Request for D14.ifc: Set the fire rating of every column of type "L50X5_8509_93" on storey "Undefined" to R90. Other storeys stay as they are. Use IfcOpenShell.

First a look at what the model holds.

```python
import ifcopenshell
import ifcopenshell.util.element

model = ifcopenshell.open("D14.ifc")
print(model.schema)
storey = next(s for s in model.by_type("IfcBuildingStorey") if s.Name == "Undefined")
columns = [e for e in ifcopenshell.util.element.get_decomposition(storey) if e.is_a("IfcColumn")]
seen = {}
for e in columns:
    element_type = ifcopenshell.util.element.get_type(e)
    key = (element_type.Name if element_type != e and element_type else None, ifcopenshell.util.element.get_pset(e, "Pset_ColumnCommon", "FireRating"))
    seen[key] = seen.get(key, 0) + 1
for (name, value), count in sorted(seen.items(), key=str):
    print(count, "x", name, "|", value)
```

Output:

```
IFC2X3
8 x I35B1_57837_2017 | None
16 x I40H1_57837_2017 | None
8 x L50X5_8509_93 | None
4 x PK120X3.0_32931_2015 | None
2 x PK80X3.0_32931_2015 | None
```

```python
import ifcopenshell
import ifcopenshell.api.pset
import ifcopenshell.util.element

model = ifcopenshell.open("D14.ifc")

storey = next(s for s in model.by_type("IfcBuildingStorey") if s.Name == "Undefined")
columns = [e for e in ifcopenshell.util.element.get_decomposition(storey) if e.is_a("IfcColumn")]

count = 0
for e in columns:
    element_type = ifcopenshell.util.element.get_type(e)
    if element_type in (None, e) or element_type.Name != "L50X5_8509_93":
        continue
    found = ifcopenshell.util.element.get_pset(e, "Pset_ColumnCommon", should_inherit=False)
    if found:
        pset = model.by_id(found["id"])
        if len(ifcopenshell.util.element.get_elements_by_pset(pset)) > 1:
            pset = ifcopenshell.api.pset.unshare_pset(model, products=[e], pset=pset)[0]
    else:
        pset = ifcopenshell.api.pset.add_pset(model, product=e, name="Pset_ColumnCommon")
    ifcopenshell.api.pset.edit_pset(model, pset=pset, properties={"FireRating": "R90"})
    count += 1

print(count, "columns updated")

model.write("D14_updated.ifc")
```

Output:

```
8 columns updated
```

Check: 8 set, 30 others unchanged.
